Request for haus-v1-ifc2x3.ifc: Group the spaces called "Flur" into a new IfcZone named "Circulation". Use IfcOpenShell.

First a look at what the model holds.

```python
import ifcopenshell

model = ifcopenshell.open("haus-v1-ifc2x3.ifc")
print(model.schema)
seen = {}
for space in model.by_type("IfcSpace"):
    seen[space.LongName] = seen.get(space.LongName, 0) + 1
for name, count in sorted(seen.items(), key=str):
    print(count, "x", name)
print("zones:", [z.Name for z in model.by_type("IfcZone")][:20])
```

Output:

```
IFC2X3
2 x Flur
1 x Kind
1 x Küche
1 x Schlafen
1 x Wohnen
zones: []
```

```python
import ifcopenshell
import ifcopenshell.api.group
import ifcopenshell.api.root

model = ifcopenshell.open("haus-v1-ifc2x3.ifc")

names = {"Flur"}
spaces = [s for s in model.by_type("IfcSpace") if s.LongName in names]

zone = ifcopenshell.api.root.create_entity(model, ifc_class="IfcZone", name="Circulation")
ifcopenshell.api.group.assign_group(model, products=spaces, group=zone)
print(len(spaces), "spaces in", zone.Name)

model.write("haus-v1-ifc2x3_edited.ifc")
```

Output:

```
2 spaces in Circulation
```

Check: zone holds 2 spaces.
